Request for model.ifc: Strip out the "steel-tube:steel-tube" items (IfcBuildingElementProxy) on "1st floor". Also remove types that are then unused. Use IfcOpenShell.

First a look at what the model holds.

```python
import ifcopenshell
import ifcopenshell.util.element

model = ifcopenshell.open("model.ifc")
print(model.schema)
storey = next(s for s in model.by_type("IfcBuildingStorey") if s.Name == "1st floor")
proxies = [e for e in ifcopenshell.util.element.get_decomposition(storey) if e.is_a("IfcBuildingElementProxy")]
seen = {}
for e in proxies:
    element_type = ifcopenshell.util.element.get_type(e)
    name = element_type.Name if element_type not in (None, e) else None
    seen[name] = seen.get(name, 0) + 1
for name, count in sorted(seen.items(), key=str):
    print(count, "x", name)
```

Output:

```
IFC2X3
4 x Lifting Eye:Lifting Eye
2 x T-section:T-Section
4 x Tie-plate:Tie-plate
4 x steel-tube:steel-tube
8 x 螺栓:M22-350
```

```python
import ifcopenshell
import ifcopenshell.api.root
import ifcopenshell.util.element

model = ifcopenshell.open("model.ifc")

storey = next(s for s in model.by_type("IfcBuildingStorey") if s.Name == "1st floor")
proxies = [e for e in ifcopenshell.util.element.get_decomposition(storey) if e.is_a("IfcBuildingElementProxy")]
targets = [e for e in proxies if (t := ifcopenshell.util.element.get_type(e)) not in (None, e) and t.Name == "steel-tube:steel-tube"]
types = {ifcopenshell.util.element.get_type(e) for e in targets} - {None, *targets}

for e in targets:
    ifcopenshell.api.root.remove_product(model, product=e)
print(len(targets), "removed")

unused = [t for t in types if not ifcopenshell.util.element.get_types(t)]
for t in unused:
    ifcopenshell.api.root.remove_product(model, product=t)
print(len(unused), "unused types removed")

model.write("model_updated.ifc")
```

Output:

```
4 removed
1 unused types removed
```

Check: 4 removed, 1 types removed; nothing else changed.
